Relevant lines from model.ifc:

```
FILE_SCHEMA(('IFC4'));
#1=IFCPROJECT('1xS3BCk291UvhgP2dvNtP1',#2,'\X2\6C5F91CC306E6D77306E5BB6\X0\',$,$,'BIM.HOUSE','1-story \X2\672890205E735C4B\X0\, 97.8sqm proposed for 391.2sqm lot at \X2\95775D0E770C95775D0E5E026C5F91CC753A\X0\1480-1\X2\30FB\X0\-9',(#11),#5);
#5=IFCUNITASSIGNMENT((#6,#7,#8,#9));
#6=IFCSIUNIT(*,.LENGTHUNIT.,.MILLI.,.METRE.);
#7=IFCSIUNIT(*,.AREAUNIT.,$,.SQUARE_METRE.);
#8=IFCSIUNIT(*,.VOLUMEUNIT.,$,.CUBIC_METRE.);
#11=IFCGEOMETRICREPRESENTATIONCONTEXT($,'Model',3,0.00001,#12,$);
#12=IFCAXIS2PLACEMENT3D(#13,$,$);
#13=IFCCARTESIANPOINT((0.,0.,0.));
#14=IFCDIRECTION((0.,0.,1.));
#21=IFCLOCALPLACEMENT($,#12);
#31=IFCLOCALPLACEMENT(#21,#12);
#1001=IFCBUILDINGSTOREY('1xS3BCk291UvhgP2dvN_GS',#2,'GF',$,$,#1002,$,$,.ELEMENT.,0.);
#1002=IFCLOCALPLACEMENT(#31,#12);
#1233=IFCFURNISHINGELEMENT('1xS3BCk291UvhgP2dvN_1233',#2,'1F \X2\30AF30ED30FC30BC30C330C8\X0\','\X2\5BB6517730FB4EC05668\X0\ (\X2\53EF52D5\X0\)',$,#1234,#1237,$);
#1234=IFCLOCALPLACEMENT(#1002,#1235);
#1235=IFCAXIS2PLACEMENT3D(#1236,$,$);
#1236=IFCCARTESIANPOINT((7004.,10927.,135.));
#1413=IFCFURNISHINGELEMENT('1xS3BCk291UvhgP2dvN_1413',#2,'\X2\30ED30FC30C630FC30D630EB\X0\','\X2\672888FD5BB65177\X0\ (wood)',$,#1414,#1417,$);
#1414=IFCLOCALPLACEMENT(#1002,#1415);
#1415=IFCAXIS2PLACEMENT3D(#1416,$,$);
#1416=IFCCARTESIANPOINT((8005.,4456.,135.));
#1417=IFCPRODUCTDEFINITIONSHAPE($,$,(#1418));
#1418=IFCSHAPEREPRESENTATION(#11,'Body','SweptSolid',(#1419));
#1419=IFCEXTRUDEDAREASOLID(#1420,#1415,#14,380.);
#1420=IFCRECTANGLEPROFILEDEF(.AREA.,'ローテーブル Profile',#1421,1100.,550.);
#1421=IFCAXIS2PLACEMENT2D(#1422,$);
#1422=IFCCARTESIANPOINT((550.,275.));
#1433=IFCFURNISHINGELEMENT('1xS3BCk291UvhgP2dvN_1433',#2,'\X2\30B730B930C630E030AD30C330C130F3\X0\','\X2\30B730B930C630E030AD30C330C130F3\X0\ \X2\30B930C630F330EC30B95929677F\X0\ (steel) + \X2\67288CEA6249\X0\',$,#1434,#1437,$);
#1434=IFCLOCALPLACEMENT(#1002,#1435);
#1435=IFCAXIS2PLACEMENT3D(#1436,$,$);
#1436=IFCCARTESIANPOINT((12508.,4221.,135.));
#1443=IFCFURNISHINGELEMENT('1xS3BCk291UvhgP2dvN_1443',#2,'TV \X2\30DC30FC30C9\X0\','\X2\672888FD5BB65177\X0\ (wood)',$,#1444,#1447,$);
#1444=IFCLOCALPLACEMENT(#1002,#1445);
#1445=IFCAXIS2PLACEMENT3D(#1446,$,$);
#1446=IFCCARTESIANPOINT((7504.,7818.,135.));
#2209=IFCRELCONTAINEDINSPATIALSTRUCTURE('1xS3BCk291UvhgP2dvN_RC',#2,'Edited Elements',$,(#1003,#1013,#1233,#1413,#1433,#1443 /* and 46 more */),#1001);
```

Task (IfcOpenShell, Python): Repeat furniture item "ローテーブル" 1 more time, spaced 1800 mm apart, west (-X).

```python
import numpy as np
import ifcopenshell
import ifcopenshell.api.geometry
import ifcopenshell.api.root
import ifcopenshell.util.element
import ifcopenshell.util.placement
import ifcopenshell.util.unit

model = ifcopenshell.open("model.ifc")
unit_scale = ifcopenshell.util.unit.calculate_unit_scale(model)


def reuse_history(source, copy):
    """copy_class also copies each property set's owner history, people and application; keep the originals."""
    for rel in copy.IsDefinedBy:
        if rel.is_a("IfcRelDefinesByProperties") and (history := rel.RelatingPropertyDefinition.OwnerHistory):
            rel.RelatingPropertyDefinition.OwnerHistory = source.OwnerHistory
            ifcopenshell.util.element.remove_deep2(model, history)


source = model.by_guid("1xS3BCk291UvhgP2dvN_1413")
base = ifcopenshell.util.placement.get_local_placement(source.ObjectPlacement)
step = np.array([-1.0, 0.0, 0.0]) * 1.8 / unit_scale

for i in range(1, 2):
    copy = ifcopenshell.api.root.copy_class(model, product=source)
    copy.Representation = ifcopenshell.util.element.copy_deep(
        model, source.Representation, exclude=["IfcGeometricRepresentationContext", "IfcRepresentationMap"]
    )
    reuse_history(source, copy)
    matrix = base.copy()
    matrix[:3, 3] += i * step
    print("added at", matrix[:3, 3].round(3) + 0.0)
    ifcopenshell.api.geometry.edit_object_placement(model, product=copy, matrix=matrix, is_si=False)

model.write("model_rev.ifc")
```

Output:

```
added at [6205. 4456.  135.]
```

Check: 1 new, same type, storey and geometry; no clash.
